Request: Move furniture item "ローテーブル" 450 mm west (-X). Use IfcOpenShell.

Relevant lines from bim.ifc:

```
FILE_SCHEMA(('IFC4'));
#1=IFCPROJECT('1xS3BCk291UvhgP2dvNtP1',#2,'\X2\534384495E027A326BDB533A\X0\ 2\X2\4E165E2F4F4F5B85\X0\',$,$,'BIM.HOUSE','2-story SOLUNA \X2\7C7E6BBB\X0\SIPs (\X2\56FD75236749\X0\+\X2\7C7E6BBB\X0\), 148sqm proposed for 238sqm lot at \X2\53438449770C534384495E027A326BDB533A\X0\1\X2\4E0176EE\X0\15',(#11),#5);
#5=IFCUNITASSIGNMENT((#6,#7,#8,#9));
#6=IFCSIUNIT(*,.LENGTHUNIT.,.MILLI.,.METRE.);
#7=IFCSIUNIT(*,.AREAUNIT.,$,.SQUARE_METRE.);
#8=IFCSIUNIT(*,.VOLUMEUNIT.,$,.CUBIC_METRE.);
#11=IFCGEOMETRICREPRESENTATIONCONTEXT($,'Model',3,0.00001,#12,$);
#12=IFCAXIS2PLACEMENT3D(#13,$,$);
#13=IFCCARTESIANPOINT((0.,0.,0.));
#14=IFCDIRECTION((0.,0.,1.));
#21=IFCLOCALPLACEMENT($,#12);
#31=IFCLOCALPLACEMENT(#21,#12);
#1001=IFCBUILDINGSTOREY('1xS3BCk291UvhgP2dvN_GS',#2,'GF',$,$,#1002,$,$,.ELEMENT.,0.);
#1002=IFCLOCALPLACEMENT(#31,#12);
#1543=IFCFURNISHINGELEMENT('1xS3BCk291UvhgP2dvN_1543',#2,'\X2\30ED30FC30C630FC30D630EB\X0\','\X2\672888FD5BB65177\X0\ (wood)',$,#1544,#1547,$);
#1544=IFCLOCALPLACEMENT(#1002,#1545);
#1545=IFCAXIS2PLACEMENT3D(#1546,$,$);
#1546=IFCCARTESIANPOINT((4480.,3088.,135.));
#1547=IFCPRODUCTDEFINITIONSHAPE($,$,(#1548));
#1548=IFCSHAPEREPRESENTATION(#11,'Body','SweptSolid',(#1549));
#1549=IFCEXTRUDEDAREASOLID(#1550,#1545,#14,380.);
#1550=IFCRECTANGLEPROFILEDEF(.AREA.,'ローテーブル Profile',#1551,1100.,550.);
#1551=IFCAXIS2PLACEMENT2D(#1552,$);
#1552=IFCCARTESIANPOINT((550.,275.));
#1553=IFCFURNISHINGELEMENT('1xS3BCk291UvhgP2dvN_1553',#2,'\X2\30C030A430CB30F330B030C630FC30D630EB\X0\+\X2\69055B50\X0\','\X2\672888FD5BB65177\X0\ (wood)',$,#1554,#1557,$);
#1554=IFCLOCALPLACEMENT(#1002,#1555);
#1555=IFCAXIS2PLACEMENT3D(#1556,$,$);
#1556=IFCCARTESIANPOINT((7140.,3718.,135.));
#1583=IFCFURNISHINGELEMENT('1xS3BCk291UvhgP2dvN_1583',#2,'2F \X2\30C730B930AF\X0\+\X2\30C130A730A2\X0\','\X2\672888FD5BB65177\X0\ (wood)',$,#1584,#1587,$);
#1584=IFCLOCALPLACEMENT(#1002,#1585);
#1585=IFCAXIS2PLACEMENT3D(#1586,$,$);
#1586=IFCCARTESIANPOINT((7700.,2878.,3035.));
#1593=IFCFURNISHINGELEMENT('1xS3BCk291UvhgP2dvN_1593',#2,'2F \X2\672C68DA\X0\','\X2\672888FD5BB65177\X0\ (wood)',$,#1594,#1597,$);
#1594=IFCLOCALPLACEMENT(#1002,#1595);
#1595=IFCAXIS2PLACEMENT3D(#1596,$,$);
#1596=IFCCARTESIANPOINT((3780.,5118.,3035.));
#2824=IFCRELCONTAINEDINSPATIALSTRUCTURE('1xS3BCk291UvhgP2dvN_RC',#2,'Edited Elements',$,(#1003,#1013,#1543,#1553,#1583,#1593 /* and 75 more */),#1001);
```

```python
import ifcopenshell
import ifcopenshell.api.geometry
import ifcopenshell.util.placement
import ifcopenshell.util.unit

model = ifcopenshell.open("bim.ifc")
unit_scale = ifcopenshell.util.unit.calculate_unit_scale(model)

item = model.by_guid("1xS3BCk291UvhgP2dvN_1543")
matrix = ifcopenshell.util.placement.get_local_placement(item.ObjectPlacement)
matrix[0, 3] -= 0.45 / unit_scale
ifcopenshell.api.geometry.edit_object_placement(model, product=item, matrix=matrix, is_si=False)

print(ifcopenshell.util.placement.get_local_placement(item.ObjectPlacement).round(3) + 0.0)

model.write("bim_edited.ifc")
```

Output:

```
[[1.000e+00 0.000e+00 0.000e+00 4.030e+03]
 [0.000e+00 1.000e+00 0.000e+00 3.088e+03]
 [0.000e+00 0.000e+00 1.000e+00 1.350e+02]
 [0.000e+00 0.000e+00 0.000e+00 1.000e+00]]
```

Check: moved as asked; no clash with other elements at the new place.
